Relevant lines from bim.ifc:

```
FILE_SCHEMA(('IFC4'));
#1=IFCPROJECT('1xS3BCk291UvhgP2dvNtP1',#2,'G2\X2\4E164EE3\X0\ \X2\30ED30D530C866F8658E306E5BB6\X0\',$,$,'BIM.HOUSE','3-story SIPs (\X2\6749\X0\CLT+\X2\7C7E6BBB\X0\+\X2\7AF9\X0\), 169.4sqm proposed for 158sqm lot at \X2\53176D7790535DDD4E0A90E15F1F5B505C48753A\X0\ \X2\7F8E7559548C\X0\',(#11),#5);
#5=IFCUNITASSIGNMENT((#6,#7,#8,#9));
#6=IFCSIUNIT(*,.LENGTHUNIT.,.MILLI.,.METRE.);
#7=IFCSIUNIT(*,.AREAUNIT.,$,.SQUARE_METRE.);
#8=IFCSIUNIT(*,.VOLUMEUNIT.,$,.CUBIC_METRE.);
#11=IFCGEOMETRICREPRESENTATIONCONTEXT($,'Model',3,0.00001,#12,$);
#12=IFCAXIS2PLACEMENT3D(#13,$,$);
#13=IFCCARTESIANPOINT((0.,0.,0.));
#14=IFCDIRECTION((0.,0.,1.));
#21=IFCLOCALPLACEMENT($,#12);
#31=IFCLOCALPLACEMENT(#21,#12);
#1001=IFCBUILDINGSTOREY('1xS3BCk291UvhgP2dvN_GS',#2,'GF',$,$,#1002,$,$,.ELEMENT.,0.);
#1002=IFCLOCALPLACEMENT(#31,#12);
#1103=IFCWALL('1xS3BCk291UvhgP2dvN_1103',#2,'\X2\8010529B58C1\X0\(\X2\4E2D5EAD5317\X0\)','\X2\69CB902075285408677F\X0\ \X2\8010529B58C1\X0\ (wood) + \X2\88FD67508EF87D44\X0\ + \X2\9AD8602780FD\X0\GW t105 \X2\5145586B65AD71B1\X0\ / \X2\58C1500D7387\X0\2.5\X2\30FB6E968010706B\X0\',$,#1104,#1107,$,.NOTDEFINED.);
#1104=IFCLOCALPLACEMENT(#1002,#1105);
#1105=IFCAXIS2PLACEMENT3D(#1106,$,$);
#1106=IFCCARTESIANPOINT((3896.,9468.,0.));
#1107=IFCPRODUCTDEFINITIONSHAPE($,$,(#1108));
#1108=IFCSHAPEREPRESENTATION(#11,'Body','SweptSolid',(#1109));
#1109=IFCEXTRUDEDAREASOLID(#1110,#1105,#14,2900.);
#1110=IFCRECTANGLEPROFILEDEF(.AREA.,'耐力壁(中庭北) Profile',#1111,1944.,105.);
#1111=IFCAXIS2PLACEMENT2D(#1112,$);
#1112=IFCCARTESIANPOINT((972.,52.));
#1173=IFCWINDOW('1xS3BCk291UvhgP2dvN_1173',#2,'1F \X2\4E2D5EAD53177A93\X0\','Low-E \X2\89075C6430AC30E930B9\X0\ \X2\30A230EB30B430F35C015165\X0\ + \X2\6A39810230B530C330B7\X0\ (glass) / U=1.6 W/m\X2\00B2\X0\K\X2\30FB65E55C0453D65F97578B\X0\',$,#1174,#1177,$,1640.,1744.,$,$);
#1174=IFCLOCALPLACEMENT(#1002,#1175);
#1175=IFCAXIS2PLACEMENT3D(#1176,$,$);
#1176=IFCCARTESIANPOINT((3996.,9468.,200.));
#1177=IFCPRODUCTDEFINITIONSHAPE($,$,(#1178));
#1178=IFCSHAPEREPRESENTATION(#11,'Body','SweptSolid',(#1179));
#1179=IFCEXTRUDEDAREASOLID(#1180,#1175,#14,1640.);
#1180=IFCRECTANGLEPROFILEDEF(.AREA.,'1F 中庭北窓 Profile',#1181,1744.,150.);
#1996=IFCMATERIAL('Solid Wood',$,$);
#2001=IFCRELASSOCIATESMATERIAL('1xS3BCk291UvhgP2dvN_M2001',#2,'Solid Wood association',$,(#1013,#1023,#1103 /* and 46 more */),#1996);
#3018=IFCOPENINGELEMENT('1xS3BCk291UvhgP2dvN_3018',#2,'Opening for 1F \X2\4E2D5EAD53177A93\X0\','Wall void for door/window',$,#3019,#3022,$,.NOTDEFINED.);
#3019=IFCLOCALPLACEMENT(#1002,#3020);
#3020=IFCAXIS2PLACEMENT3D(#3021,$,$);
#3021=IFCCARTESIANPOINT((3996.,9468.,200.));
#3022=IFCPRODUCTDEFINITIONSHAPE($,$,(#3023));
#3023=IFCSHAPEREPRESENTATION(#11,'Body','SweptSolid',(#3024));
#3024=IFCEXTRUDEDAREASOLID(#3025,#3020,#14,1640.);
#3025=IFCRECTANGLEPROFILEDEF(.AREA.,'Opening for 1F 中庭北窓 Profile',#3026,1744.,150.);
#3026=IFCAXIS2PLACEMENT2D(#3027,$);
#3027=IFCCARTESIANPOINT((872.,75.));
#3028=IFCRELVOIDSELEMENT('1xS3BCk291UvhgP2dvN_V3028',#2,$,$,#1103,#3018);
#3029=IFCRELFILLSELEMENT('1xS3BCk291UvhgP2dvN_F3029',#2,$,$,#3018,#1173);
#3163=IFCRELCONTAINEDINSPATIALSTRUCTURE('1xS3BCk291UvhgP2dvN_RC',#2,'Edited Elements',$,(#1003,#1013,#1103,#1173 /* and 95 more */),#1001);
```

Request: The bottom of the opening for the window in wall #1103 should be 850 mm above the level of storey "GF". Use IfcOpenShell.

```python
import numpy as np
import ifcopenshell
import ifcopenshell.api.geometry
import ifcopenshell.geom
import ifcopenshell.util.element
import ifcopenshell.util.placement
import ifcopenshell.util.shape
import ifcopenshell.util.unit

model = ifcopenshell.open("bim.ifc")
unit_scale = ifcopenshell.util.unit.calculate_unit_scale(model)

window = model.by_id(1173)
opening = window.FillsVoids[0].RelatingOpeningElement
storey = ifcopenshell.util.element.get_container(window, ifc_class="IfcBuildingStorey")
level = ifcopenshell.util.placement.get_local_placement(storey.ObjectPlacement)[2, 3]

# The opening's origin need not be at the sill, so measure its lowest point.
shape = ifcopenshell.geom.create_shape(ifcopenshell.geom.settings(), opening)
bottom = ifcopenshell.util.shape.get_shape_bottom_elevation(shape, shape.geometry) / unit_scale
dz = level + 0.85 / unit_scale - bottom

shift = np.array([0.0, 0.0, dz])
# The window is not placed relative to its opening, so move both.
for product in (opening, window):
    matrix = ifcopenshell.util.placement.get_local_placement(product.ObjectPlacement)
    matrix[:3, 3] += shift
    ifcopenshell.api.geometry.edit_object_placement(model, product=product, matrix=matrix, is_si=False)

print(f"moved by {dz * unit_scale:+.3f} m")

model.write("bim_rev.ifc")
```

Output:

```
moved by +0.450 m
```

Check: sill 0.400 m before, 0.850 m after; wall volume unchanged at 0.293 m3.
